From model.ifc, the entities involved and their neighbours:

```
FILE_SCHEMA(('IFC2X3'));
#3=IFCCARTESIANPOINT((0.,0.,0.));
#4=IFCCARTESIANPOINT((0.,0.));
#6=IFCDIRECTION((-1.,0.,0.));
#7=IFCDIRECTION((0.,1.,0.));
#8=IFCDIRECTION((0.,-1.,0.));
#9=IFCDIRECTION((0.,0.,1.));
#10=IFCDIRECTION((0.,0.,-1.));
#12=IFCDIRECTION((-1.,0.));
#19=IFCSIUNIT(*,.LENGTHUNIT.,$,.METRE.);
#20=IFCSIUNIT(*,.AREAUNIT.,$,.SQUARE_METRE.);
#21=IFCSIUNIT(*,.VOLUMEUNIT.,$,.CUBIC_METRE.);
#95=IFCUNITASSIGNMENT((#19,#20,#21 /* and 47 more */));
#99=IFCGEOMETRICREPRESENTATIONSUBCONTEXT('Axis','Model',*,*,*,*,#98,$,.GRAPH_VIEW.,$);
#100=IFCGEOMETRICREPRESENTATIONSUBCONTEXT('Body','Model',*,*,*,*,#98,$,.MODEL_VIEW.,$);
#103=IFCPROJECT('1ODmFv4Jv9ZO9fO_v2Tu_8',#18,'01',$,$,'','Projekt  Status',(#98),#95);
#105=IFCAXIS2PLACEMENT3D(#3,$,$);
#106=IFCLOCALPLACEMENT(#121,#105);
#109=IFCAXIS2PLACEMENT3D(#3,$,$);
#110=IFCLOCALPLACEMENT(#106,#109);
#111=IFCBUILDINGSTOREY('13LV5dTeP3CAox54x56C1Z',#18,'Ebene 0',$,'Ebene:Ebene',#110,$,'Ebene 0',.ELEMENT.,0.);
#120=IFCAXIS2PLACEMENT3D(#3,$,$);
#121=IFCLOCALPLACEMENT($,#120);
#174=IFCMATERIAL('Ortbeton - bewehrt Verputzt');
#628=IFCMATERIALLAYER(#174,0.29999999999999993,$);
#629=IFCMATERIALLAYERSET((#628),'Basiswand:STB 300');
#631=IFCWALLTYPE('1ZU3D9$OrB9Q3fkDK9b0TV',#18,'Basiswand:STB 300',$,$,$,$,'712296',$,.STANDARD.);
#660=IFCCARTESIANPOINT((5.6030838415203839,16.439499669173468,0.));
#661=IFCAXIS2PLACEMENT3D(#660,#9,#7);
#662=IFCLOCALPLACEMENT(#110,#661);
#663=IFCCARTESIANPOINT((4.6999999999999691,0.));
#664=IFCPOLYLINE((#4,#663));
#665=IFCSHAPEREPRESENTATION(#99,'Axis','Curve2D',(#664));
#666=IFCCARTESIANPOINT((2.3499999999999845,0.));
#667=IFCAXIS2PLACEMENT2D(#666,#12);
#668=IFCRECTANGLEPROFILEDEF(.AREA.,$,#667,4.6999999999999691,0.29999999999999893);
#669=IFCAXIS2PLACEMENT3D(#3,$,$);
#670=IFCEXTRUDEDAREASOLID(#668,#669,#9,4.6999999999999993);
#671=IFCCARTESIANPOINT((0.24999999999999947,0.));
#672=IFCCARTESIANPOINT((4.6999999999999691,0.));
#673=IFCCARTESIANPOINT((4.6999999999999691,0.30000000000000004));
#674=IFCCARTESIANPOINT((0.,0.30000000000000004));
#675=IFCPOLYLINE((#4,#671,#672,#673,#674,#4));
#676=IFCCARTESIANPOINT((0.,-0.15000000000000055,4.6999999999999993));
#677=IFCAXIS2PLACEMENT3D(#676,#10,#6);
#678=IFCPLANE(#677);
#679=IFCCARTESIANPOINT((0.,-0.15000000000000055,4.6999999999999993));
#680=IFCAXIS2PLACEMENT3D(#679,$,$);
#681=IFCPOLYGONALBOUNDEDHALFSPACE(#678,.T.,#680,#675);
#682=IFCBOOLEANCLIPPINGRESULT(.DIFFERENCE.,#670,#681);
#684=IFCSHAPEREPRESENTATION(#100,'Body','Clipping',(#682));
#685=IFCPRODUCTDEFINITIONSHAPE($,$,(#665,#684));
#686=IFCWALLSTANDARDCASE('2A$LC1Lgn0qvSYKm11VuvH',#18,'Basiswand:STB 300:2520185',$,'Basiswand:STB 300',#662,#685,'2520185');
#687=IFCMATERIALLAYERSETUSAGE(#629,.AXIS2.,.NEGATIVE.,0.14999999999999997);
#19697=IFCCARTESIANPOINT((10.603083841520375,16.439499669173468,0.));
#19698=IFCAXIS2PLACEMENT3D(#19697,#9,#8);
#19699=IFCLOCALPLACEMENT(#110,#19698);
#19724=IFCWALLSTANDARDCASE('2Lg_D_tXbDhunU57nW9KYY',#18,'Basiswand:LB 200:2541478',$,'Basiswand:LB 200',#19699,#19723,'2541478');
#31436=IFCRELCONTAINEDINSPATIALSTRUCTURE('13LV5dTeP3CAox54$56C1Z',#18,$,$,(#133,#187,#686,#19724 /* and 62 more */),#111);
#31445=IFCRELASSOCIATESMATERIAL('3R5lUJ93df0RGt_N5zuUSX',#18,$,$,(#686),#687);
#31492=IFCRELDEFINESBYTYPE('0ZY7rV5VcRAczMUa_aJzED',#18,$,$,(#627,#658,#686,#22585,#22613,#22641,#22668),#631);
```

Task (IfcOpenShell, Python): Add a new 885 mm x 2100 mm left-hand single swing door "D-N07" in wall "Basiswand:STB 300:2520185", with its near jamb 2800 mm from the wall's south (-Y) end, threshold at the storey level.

```python
import numpy as np
import ifcopenshell
import ifcopenshell.api.feature
import ifcopenshell.api.geometry
import ifcopenshell.api.root
import ifcopenshell.api.spatial
import ifcopenshell.api.type
import ifcopenshell.geom
import ifcopenshell.util.element
import ifcopenshell.util.placement
import ifcopenshell.util.representation
import ifcopenshell.util.shape
import ifcopenshell.util.unit

model = ifcopenshell.open("model.ifc")
unit_scale = ifcopenshell.util.unit.calculate_unit_scale(model)
settings = ifcopenshell.geom.settings()


def volume(element):
    """Net volume in cubic metres, openings subtracted."""
    shape = ifcopenshell.geom.create_shape(settings, element)
    return ifcopenshell.util.shape.get_volume(shape.geometry)


wall = model.by_guid("2A$LC1Lgn0qvSYKm11VuvH")
storey = ifcopenshell.util.element.get_container(wall, ifc_class="IfcBuildingStorey")
context = ifcopenshell.util.representation.get_context(model, "Model", "Body", "MODEL_VIEW")
before = volume(wall)

width, height, from_end, sill = 0.885, 2.1, 2.8, 0.0  # metres

# The wall runs along its own X axis, and the end named is its -X end.
wall_shape = ifcopenshell.geom.create_shape(settings, wall)
x, y, z = ifcopenshell.util.shape.get_vertices(wall_shape.geometry).T
start = x.min() + from_end
face, thickness = float(y.min()), float(y.max() - y.min())
wall_matrix = ifcopenshell.util.placement.get_local_placement(wall.ObjectPlacement)
level = ifcopenshell.util.placement.get_local_placement(storey.ObjectPlacement)[2, 3]


def in_wall(x, y):
    """Placement at x, y metres in the wall's axes, at sill height."""
    matrix = wall_matrix.copy()
    matrix[:, 3] = wall_matrix @ np.array([x / unit_scale, y / unit_scale, 0.0, 1.0])
    matrix[2, 3] = level + sill / unit_scale
    return matrix


# Opening: a box that overshoots both wall faces by 50 mm.
opening = ifcopenshell.api.root.create_entity(model, ifc_class="IfcOpeningElement")
box = ifcopenshell.api.geometry.add_wall_representation(
    model, context=context, length=width, height=height, thickness=thickness + 0.1
)
ifcopenshell.api.geometry.assign_representation(model, product=opening, representation=box)
ifcopenshell.api.geometry.edit_object_placement(model, product=opening, matrix=in_wall(start, face - 0.05), is_si=False)
ifcopenshell.api.feature.add_feature(model, feature=opening, element=wall)

door = ifcopenshell.api.root.create_entity(model, ifc_class="IfcDoor", name="D-N07")
door.OverallWidth, door.OverallHeight = width / unit_scale, height / unit_scale
body = ifcopenshell.api.geometry.add_door_representation(
    model,
    context=context,
    overall_width=door.OverallWidth,
    overall_height=door.OverallHeight,
    operation_type="SINGLE_SWING_LEFT",
    lining_properties={"LiningDepth": thickness / unit_scale, "ThresholdDepth": thickness / unit_scale},
)
ifcopenshell.api.geometry.assign_representation(model, product=door, representation=body)
ifcopenshell.api.spatial.assign_container(model, products=[door], relating_structure=storey)
fills = ifcopenshell.api.feature.add_filling(model, opening=opening, element=door)
fills.OwnerHistory = door.OwnerHistory  # required in IFC2X3

# IFC2X3 keeps the operation on the door style.
style = ifcopenshell.api.root.create_entity(model, ifc_class="IfcDoorStyle", name="D-N07")
style.OperationType, style.ConstructionType = "SINGLE_SWING_LEFT", "NOTDEFINED"
style.ParameterTakesPrecedence = style.Sizeable = False
ifcopenshell.api.type.assign_type(model, related_objects=[door], relating_type=style)

# The lining spans the wall, so the door starts at the wall face.
ifcopenshell.api.geometry.edit_object_placement(model, product=door, matrix=in_wall(start, face), is_si=False)

after = volume(wall)

print(f"wall volume {before:.3f} -> {after:.3f} m3")

model.write("model-out.ifc")
```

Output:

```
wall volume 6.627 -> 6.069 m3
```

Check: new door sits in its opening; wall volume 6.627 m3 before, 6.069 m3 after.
